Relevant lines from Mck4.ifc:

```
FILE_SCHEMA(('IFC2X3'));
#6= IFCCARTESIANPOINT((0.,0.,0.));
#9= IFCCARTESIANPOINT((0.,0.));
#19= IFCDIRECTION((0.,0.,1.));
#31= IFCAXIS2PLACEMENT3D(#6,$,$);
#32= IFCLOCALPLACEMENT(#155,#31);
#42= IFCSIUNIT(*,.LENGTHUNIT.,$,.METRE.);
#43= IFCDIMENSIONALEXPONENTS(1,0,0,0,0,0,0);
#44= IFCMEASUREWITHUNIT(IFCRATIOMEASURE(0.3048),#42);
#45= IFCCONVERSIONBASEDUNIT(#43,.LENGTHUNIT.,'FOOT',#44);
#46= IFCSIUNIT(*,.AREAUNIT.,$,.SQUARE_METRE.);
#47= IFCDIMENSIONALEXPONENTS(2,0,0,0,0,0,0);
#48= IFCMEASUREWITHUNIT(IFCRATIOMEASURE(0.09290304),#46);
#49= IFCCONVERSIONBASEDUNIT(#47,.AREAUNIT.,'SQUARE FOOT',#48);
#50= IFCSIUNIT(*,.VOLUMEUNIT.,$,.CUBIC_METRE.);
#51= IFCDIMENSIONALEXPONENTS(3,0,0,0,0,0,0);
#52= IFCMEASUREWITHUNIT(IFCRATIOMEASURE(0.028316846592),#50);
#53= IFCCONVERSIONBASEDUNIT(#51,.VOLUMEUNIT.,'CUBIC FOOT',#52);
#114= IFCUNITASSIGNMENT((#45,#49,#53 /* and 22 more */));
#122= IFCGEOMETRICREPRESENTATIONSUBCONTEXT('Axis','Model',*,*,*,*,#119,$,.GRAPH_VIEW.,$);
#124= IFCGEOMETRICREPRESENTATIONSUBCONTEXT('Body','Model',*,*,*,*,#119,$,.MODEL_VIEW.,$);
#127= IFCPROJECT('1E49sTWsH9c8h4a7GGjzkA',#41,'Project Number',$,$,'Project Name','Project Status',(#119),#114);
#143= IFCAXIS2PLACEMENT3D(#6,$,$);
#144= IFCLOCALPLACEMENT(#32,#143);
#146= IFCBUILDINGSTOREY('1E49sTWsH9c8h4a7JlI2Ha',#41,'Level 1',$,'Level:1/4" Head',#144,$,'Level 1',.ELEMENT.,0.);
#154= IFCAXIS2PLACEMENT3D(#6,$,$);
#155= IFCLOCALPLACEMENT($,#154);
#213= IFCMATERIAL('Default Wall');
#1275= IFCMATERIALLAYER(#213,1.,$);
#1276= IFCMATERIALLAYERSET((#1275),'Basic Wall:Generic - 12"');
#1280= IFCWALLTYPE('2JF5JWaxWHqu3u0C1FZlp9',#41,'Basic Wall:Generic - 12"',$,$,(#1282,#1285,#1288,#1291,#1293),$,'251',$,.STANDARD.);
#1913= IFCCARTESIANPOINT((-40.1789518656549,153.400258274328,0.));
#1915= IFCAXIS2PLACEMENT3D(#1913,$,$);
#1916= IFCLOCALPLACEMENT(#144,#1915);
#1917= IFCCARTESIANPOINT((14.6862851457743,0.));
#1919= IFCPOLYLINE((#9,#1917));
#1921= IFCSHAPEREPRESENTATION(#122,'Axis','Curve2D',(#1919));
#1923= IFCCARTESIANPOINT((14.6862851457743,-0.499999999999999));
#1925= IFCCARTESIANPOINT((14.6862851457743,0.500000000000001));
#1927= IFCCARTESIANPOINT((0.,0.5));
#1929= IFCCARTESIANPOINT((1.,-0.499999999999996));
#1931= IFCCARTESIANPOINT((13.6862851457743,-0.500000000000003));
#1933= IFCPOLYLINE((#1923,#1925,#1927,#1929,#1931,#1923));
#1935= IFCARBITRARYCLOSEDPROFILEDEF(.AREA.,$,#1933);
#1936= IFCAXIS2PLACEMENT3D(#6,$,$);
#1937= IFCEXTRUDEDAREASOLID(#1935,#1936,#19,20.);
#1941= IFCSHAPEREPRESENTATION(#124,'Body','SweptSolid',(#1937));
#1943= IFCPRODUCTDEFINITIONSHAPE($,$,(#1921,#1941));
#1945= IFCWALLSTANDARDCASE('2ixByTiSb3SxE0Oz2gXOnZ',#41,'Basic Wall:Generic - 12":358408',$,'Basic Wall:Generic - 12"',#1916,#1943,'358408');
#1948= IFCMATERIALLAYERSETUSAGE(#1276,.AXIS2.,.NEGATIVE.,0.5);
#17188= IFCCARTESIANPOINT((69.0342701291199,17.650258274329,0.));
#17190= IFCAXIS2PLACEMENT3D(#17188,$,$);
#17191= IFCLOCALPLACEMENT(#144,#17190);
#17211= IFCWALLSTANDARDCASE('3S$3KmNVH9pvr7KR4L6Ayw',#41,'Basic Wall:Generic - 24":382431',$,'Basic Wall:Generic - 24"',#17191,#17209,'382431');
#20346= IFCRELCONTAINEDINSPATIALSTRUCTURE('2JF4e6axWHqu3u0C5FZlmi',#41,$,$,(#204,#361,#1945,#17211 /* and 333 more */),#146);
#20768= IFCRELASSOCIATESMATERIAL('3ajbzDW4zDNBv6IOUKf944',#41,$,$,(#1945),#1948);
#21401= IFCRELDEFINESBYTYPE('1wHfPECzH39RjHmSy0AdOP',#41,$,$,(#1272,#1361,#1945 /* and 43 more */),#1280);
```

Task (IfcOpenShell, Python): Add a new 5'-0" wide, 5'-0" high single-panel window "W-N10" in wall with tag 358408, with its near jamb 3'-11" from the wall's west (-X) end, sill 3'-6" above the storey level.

```python
import numpy as np
import ifcopenshell
import ifcopenshell.api.feature
import ifcopenshell.api.geometry
import ifcopenshell.api.root
import ifcopenshell.api.spatial
import ifcopenshell.api.type
import ifcopenshell.geom
import ifcopenshell.util.element
import ifcopenshell.util.placement
import ifcopenshell.util.representation
import ifcopenshell.util.shape
import ifcopenshell.util.unit

model = ifcopenshell.open("Mck4.ifc")
unit_scale = ifcopenshell.util.unit.calculate_unit_scale(model)
settings = ifcopenshell.geom.settings()


def volume(element):
    """Net volume in cubic metres, openings subtracted."""
    shape = ifcopenshell.geom.create_shape(settings, element)
    return ifcopenshell.util.shape.get_volume(shape.geometry)


wall = model.by_guid("2ixByTiSb3SxE0Oz2gXOnZ")
storey = ifcopenshell.util.element.get_container(wall, ifc_class="IfcBuildingStorey")
context = ifcopenshell.util.representation.get_context(model, "Model", "Body", "MODEL_VIEW")
before = volume(wall)

width, height, from_end, sill = 1.524, 1.524, 1.1938, 1.0668  # metres

# The wall runs along its own X axis, and the end named is its -X end.
wall_shape = ifcopenshell.geom.create_shape(settings, wall)
x, y, z = ifcopenshell.util.shape.get_vertices(wall_shape.geometry).T
start = x.min() + from_end
face, thickness = float(y.min()), float(y.max() - y.min())
wall_matrix = ifcopenshell.util.placement.get_local_placement(wall.ObjectPlacement)
level = ifcopenshell.util.placement.get_local_placement(storey.ObjectPlacement)[2, 3]


def in_wall(x, y):
    """Placement at x, y metres in the wall's axes, at sill height."""
    matrix = wall_matrix.copy()
    matrix[:, 3] = wall_matrix @ np.array([x / unit_scale, y / unit_scale, 0.0, 1.0])
    matrix[2, 3] = level + sill / unit_scale
    return matrix


# Opening: a box that overshoots both wall faces by 50 mm.
opening = ifcopenshell.api.root.create_entity(model, ifc_class="IfcOpeningElement")
box = ifcopenshell.api.geometry.add_wall_representation(
    model, context=context, length=width, height=height, thickness=thickness + 0.1
)
ifcopenshell.api.geometry.assign_representation(model, product=opening, representation=box)
ifcopenshell.api.geometry.edit_object_placement(model, product=opening, matrix=in_wall(start, face - 0.05), is_si=False)
ifcopenshell.api.feature.add_feature(model, feature=opening, element=wall)

window = ifcopenshell.api.root.create_entity(model, ifc_class="IfcWindow", name="W-N10")
window.OverallWidth, window.OverallHeight = width / unit_scale, height / unit_scale
body = ifcopenshell.api.geometry.add_window_representation(
    model,
    context=context,
    overall_width=window.OverallWidth,
    overall_height=window.OverallHeight,
    partition_type="SINGLE_PANEL",
)
ifcopenshell.api.geometry.assign_representation(model, product=window, representation=body)
ifcopenshell.api.spatial.assign_container(model, products=[window], relating_structure=storey)
fills = ifcopenshell.api.feature.add_filling(model, opening=opening, element=window)
fills.OwnerHistory = window.OwnerHistory  # required in IFC2X3

# IFC2X3 keeps the operation on the window style.
style = ifcopenshell.api.root.create_entity(model, ifc_class="IfcWindowStyle", name="W-N10")
style.OperationType, style.ConstructionType = "SINGLE_PANEL", "NOTDEFINED"
style.ParameterTakesPrecedence = style.Sizeable = False
ifcopenshell.api.type.assign_type(model, related_objects=[window], relating_type=style)

# Centre the window in the wall's thickness.
ifcopenshell.api.geometry.edit_object_placement(model, product=window, matrix=in_wall(start, face), is_si=False)
window_shape = ifcopenshell.geom.create_shape(settings, window)
depth = ifcopenshell.util.shape.get_vertices(window_shape.geometry)[:, 1]
offset = face + thickness / 2 - (depth.min() + depth.max()) / 2
ifcopenshell.api.geometry.edit_object_placement(model, product=window, matrix=in_wall(start, offset), is_si=False)

after = volume(wall)

print(f"wall volume {before:.3f} -> {after:.3f} m3")

model.write("Mck4_rev.ifc")
```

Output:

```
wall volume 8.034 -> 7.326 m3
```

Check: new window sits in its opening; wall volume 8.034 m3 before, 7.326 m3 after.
